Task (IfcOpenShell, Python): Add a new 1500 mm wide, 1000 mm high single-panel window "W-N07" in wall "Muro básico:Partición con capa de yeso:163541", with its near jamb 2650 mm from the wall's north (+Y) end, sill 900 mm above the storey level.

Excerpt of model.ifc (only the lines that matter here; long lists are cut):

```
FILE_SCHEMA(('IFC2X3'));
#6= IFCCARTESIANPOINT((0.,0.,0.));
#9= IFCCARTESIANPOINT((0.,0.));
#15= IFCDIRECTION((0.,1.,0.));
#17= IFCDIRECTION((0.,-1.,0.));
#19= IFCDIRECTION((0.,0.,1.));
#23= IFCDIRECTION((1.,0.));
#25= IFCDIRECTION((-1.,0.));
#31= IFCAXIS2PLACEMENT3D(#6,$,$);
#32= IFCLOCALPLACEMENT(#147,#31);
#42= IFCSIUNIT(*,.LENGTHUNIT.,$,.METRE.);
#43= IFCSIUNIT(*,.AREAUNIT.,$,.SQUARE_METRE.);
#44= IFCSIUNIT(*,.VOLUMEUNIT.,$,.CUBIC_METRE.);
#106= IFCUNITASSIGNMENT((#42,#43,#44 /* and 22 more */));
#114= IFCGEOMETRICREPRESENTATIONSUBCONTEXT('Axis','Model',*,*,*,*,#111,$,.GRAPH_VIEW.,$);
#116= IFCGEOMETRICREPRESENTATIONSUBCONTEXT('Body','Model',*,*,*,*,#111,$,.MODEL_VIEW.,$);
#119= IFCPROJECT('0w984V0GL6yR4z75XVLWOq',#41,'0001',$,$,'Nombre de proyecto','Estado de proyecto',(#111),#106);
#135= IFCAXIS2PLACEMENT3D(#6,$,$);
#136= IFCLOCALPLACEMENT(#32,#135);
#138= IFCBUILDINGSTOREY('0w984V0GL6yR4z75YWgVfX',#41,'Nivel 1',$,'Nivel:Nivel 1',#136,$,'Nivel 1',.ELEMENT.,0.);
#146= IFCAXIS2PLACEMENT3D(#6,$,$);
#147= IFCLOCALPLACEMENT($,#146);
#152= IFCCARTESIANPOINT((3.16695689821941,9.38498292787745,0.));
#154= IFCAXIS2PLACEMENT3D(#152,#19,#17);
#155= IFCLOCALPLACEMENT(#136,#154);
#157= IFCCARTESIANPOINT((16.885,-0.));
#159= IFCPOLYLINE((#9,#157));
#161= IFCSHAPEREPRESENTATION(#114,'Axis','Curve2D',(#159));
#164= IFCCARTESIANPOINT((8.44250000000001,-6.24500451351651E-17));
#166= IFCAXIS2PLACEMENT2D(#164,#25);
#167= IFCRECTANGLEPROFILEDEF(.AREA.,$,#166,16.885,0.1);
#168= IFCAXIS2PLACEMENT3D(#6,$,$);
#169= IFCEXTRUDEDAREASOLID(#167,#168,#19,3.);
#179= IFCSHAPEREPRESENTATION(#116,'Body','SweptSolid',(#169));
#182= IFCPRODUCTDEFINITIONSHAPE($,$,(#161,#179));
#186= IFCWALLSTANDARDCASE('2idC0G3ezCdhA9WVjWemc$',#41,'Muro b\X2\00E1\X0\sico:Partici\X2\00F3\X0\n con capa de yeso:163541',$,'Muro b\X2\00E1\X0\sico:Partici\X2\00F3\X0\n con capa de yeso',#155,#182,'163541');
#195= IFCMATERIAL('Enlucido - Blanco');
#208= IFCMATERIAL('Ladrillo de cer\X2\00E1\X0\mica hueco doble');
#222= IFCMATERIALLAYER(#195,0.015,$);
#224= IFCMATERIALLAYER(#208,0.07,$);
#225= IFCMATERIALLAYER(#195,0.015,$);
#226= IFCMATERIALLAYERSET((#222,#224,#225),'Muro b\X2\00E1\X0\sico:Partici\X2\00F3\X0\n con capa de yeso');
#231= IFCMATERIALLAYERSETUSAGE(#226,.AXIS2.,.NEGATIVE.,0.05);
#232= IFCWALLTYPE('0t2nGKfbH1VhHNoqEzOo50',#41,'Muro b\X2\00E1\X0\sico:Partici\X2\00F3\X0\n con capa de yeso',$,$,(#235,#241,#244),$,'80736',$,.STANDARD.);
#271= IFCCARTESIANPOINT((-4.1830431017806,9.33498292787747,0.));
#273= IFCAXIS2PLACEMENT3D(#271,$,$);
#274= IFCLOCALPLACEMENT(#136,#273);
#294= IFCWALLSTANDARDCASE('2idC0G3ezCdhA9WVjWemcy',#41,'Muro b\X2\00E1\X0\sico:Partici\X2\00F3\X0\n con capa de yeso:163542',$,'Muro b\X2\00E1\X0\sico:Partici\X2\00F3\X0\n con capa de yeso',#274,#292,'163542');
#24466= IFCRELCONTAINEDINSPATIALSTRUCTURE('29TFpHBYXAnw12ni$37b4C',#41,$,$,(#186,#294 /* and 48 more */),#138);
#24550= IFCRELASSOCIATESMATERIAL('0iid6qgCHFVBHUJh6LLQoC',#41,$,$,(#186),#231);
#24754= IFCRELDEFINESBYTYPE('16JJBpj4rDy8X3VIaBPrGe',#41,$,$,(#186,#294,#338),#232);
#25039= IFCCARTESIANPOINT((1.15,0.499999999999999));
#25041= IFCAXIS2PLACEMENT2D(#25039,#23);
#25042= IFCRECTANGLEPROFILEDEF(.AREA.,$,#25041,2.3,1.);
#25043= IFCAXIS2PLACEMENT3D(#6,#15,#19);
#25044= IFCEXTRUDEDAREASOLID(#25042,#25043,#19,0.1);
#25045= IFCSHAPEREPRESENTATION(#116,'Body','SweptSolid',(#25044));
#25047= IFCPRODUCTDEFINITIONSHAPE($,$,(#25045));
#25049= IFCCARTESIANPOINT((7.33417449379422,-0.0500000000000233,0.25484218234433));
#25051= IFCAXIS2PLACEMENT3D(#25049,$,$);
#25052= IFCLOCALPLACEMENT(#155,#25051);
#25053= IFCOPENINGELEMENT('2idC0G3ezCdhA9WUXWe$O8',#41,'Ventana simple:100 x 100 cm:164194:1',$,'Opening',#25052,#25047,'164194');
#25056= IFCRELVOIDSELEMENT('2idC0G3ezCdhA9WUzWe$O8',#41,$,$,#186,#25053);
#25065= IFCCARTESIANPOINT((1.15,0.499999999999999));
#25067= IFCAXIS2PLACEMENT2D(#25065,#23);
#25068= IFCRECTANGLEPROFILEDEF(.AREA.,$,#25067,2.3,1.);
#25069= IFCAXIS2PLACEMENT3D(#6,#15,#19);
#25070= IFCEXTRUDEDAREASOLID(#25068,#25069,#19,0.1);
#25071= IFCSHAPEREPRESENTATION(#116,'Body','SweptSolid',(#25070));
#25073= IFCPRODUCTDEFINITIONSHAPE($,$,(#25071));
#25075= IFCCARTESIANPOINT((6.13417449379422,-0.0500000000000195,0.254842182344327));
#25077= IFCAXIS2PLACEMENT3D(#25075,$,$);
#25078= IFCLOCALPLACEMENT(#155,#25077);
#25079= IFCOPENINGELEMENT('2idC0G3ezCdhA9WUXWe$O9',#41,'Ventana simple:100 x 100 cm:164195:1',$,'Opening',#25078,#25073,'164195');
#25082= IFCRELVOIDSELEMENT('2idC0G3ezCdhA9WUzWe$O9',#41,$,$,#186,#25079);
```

```python
import numpy as np
import ifcopenshell
import ifcopenshell.api.feature
import ifcopenshell.api.geometry
import ifcopenshell.api.root
import ifcopenshell.api.spatial
import ifcopenshell.api.type
import ifcopenshell.geom
import ifcopenshell.util.element
import ifcopenshell.util.placement
import ifcopenshell.util.representation
import ifcopenshell.util.shape
import ifcopenshell.util.unit

model = ifcopenshell.open("model.ifc")
unit_scale = ifcopenshell.util.unit.calculate_unit_scale(model)
settings = ifcopenshell.geom.settings()


def volume(element):
    """Net volume in cubic metres, openings subtracted."""
    shape = ifcopenshell.geom.create_shape(settings, element)
    return ifcopenshell.util.shape.get_volume(shape.geometry)


wall = model.by_id(186)
storey = ifcopenshell.util.element.get_container(wall, ifc_class="IfcBuildingStorey")
context = ifcopenshell.util.representation.get_context(model, "Model", "Body", "MODEL_VIEW")
before = volume(wall)

width, height, from_end, sill = 1.5, 1, 2.65, 0.9  # metres

# The wall runs along its own X axis, and the end named is its -X end.
wall_shape = ifcopenshell.geom.create_shape(settings, wall)
x, y, z = ifcopenshell.util.shape.get_vertices(wall_shape.geometry).T
start = x.min() + from_end
face, thickness = float(y.min()), float(y.max() - y.min())
wall_matrix = ifcopenshell.util.placement.get_local_placement(wall.ObjectPlacement)
level = ifcopenshell.util.placement.get_local_placement(storey.ObjectPlacement)[2, 3]


def in_wall(x, y):
    """Placement at x, y metres in the wall's axes, at sill height."""
    matrix = wall_matrix.copy()
    matrix[:, 3] = wall_matrix @ np.array([x / unit_scale, y / unit_scale, 0.0, 1.0])
    matrix[2, 3] = level + sill / unit_scale
    return matrix


# Opening: a box that overshoots both wall faces by 50 mm.
opening = ifcopenshell.api.root.create_entity(model, ifc_class="IfcOpeningElement")
box = ifcopenshell.api.geometry.add_wall_representation(
    model, context=context, length=width, height=height, thickness=thickness + 0.1
)
ifcopenshell.api.geometry.assign_representation(model, product=opening, representation=box)
ifcopenshell.api.geometry.edit_object_placement(model, product=opening, matrix=in_wall(start, face - 0.05), is_si=False)
ifcopenshell.api.feature.add_feature(model, feature=opening, element=wall)

window = ifcopenshell.api.root.create_entity(model, ifc_class="IfcWindow", name="W-N07")
window.OverallWidth, window.OverallHeight = width / unit_scale, height / unit_scale
body = ifcopenshell.api.geometry.add_window_representation(
    model,
    context=context,
    overall_width=window.OverallWidth,
    overall_height=window.OverallHeight,
    partition_type="SINGLE_PANEL",
)
ifcopenshell.api.geometry.assign_representation(model, product=window, representation=body)
ifcopenshell.api.spatial.assign_container(model, products=[window], relating_structure=storey)
fills = ifcopenshell.api.feature.add_filling(model, opening=opening, element=window)
fills.OwnerHistory = window.OwnerHistory  # required in IFC2X3

# IFC2X3 keeps the operation on the window style.
style = ifcopenshell.api.root.create_entity(model, ifc_class="IfcWindowStyle", name="W-N07")
style.OperationType, style.ConstructionType = "SINGLE_PANEL", "NOTDEFINED"
style.ParameterTakesPrecedence = style.Sizeable = False
ifcopenshell.api.type.assign_type(model, related_objects=[window], relating_type=style)

# Centre the window in the wall's thickness.
ifcopenshell.api.geometry.edit_object_placement(model, product=window, matrix=in_wall(start, face), is_si=False)
window_shape = ifcopenshell.geom.create_shape(settings, window)
depth = ifcopenshell.util.shape.get_vertices(window_shape.geometry)[:, 1]
offset = face + thickness / 2 - (depth.min() + depth.max()) / 2
ifcopenshell.api.geometry.edit_object_placement(model, product=window, matrix=in_wall(start, offset), is_si=False)

after = volume(wall)

print(f"wall volume {before:.3f} -> {after:.3f} m3")

model.write("model_rev.ifc")
```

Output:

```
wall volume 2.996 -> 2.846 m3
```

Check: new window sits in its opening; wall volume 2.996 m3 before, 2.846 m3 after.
